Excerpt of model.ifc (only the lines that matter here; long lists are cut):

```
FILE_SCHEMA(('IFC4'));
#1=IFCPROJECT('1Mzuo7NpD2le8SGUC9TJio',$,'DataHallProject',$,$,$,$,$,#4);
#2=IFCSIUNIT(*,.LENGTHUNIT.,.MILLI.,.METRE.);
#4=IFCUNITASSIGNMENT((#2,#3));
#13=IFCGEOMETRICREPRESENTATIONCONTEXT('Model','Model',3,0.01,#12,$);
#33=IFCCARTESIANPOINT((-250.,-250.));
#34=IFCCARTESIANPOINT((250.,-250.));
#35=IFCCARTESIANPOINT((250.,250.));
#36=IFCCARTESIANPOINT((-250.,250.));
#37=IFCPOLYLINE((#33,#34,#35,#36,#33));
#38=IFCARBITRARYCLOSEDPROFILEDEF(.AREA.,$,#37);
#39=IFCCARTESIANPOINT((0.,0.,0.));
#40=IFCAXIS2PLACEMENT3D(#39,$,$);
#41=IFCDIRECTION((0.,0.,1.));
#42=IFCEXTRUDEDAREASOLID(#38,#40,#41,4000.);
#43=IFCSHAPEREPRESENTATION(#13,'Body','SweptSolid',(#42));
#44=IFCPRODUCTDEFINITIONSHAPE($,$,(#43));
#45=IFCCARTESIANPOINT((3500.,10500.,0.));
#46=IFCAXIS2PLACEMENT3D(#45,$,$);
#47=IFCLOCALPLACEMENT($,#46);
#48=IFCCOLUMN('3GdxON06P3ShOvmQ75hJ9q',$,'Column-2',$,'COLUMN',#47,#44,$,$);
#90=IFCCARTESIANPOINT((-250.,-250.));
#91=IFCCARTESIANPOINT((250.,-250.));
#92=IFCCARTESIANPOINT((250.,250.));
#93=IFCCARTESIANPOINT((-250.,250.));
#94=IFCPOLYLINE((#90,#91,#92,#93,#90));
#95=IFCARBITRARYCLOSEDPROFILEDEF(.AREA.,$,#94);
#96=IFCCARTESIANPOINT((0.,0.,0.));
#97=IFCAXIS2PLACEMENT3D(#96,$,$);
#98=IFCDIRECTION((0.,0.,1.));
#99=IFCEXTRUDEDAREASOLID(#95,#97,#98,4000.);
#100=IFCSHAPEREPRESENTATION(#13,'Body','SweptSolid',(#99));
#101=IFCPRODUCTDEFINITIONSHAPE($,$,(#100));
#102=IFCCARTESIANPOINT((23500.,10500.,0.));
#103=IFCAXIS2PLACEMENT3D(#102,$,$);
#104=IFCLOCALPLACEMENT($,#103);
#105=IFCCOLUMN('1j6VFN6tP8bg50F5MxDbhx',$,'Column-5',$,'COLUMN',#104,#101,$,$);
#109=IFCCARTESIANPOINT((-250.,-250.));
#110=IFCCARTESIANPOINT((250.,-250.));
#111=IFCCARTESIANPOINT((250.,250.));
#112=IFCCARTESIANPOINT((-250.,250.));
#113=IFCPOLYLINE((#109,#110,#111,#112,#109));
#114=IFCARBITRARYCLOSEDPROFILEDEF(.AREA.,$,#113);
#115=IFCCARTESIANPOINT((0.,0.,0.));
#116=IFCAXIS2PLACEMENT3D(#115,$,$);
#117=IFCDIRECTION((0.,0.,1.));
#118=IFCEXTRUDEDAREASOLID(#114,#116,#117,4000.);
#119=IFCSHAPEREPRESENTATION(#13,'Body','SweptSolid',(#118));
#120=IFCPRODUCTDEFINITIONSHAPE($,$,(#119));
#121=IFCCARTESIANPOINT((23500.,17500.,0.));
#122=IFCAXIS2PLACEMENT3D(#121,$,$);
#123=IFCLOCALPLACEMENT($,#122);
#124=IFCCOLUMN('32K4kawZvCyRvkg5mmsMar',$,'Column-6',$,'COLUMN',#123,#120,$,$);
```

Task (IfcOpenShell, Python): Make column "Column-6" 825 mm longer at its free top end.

```python
import ifcopenshell
import ifcopenshell.util.unit

model = ifcopenshell.open("model.ifc")
unit_scale = ifcopenshell.util.unit.calculate_unit_scale(model)

member = model.by_guid("32K4kawZvCyRvkg5mmsMar")
change = 0.825 / unit_scale

# The extrusion runs towards the end named, so only its depth changes.
body = next(r for r in member.Representation.Representations if r.RepresentationIdentifier == "Body")
solid = body.Items[0]
old_length = solid.Depth
solid.Depth += change

print(f"length {old_length:g} -> {solid.Depth:g}")

model.write("model_v2.ifc")
```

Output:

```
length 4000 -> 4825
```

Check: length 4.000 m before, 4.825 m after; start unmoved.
